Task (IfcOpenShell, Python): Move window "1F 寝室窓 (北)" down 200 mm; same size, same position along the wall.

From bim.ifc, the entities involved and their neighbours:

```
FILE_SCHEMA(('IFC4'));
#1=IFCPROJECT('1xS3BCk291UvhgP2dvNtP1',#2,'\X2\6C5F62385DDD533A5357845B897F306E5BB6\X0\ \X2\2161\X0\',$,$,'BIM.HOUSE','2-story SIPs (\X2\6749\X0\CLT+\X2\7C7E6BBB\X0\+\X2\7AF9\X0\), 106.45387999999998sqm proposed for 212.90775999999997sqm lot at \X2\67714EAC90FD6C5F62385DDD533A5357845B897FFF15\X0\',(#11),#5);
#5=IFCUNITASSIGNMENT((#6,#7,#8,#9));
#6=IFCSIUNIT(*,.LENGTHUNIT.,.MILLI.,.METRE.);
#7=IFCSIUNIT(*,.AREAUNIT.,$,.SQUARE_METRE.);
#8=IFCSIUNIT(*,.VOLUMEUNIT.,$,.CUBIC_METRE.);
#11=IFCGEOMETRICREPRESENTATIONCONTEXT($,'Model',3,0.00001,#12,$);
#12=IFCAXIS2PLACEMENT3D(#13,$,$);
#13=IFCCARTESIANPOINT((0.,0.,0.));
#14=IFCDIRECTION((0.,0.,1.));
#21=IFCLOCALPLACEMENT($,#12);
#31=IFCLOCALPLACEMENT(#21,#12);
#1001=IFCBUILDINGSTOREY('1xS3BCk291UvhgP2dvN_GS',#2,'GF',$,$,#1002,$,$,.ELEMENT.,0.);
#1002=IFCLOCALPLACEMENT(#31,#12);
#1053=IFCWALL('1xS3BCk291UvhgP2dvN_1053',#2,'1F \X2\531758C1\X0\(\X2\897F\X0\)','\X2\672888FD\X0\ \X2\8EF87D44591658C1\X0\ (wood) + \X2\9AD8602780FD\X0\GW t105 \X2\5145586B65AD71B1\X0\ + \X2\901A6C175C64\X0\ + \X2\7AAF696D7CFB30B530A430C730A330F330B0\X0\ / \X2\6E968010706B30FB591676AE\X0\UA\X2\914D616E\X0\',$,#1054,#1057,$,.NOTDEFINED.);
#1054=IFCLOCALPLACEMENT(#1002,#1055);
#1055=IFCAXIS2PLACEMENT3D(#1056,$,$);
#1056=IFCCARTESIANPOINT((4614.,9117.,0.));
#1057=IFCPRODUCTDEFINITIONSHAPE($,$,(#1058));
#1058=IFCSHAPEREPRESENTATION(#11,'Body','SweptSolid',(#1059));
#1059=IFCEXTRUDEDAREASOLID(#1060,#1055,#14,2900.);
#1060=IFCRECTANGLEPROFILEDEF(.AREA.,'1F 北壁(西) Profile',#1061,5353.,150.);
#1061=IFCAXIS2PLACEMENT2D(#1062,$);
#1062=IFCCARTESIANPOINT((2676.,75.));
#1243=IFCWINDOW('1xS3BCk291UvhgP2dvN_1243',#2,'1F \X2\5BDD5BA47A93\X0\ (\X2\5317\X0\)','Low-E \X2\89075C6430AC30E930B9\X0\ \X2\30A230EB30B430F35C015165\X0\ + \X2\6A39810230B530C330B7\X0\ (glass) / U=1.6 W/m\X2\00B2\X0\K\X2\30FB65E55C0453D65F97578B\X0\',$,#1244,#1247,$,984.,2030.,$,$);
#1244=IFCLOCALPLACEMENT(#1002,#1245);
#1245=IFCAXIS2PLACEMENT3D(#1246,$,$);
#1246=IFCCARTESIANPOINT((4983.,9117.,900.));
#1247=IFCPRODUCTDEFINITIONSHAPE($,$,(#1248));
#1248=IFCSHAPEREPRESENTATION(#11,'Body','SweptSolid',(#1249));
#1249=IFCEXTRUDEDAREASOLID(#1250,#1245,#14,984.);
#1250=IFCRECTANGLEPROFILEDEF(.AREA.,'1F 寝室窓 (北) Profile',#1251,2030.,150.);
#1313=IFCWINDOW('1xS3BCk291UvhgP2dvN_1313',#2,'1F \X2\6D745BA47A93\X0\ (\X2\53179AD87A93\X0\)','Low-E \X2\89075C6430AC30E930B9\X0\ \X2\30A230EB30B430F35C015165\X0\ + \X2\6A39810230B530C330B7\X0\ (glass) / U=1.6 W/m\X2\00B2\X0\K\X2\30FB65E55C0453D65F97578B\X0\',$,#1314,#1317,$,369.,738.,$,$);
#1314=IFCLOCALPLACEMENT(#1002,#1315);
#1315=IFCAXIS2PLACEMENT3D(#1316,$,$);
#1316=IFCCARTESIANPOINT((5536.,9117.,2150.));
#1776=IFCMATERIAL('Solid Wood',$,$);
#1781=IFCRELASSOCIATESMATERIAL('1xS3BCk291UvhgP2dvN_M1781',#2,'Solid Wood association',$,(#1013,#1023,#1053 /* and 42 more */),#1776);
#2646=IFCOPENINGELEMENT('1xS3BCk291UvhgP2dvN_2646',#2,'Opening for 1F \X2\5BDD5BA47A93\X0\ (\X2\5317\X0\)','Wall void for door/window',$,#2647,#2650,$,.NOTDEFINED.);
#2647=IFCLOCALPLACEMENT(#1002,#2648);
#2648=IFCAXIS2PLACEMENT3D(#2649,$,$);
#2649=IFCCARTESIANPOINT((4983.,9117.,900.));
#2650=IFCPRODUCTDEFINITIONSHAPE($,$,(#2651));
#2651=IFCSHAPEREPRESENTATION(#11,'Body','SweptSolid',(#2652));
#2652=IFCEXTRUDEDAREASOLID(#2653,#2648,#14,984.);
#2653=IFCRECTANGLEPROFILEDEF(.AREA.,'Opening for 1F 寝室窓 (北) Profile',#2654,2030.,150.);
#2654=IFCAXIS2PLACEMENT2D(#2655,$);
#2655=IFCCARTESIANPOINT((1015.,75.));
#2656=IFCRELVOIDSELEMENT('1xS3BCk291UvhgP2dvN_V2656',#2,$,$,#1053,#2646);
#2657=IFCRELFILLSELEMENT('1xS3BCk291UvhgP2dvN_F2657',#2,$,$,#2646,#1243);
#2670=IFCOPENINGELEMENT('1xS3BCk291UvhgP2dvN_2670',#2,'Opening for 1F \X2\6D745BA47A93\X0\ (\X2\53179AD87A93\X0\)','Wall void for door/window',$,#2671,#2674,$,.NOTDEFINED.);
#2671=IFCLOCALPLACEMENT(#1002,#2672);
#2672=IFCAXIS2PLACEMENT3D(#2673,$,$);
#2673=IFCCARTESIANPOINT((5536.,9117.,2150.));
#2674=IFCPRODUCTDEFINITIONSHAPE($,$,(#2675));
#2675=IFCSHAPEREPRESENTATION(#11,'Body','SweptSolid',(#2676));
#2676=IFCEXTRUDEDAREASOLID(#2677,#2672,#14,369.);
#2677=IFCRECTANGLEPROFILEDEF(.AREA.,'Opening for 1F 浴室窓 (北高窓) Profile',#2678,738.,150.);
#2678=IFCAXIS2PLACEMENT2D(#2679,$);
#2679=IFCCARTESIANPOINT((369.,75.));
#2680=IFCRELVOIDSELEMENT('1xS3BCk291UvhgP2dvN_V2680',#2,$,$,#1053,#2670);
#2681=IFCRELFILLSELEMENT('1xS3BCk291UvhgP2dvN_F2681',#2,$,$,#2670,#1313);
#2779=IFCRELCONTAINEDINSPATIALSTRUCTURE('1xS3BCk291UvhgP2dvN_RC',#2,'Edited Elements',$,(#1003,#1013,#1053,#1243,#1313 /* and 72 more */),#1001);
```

```python
import numpy as np
import ifcopenshell
import ifcopenshell.api.geometry
import ifcopenshell.util.placement
import ifcopenshell.util.unit

model = ifcopenshell.open("bim.ifc")
unit_scale = ifcopenshell.util.unit.calculate_unit_scale(model)

window = model.by_guid("1xS3BCk291UvhgP2dvN_1243")
opening = window.FillsVoids[0].RelatingOpeningElement
dz = -200.0

shift = np.array([0.0, 0.0, dz])
# The window is not placed relative to its opening, so move both.
for product in (opening, window):
    matrix = ifcopenshell.util.placement.get_local_placement(product.ObjectPlacement)
    matrix[:3, 3] += shift
    ifcopenshell.api.geometry.edit_object_placement(model, product=product, matrix=matrix, is_si=False)

print(f"moved by {dz * unit_scale:+.3f} m")

model.write("bim_updated.ifc")
```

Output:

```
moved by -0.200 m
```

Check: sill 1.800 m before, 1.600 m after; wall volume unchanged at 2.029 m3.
